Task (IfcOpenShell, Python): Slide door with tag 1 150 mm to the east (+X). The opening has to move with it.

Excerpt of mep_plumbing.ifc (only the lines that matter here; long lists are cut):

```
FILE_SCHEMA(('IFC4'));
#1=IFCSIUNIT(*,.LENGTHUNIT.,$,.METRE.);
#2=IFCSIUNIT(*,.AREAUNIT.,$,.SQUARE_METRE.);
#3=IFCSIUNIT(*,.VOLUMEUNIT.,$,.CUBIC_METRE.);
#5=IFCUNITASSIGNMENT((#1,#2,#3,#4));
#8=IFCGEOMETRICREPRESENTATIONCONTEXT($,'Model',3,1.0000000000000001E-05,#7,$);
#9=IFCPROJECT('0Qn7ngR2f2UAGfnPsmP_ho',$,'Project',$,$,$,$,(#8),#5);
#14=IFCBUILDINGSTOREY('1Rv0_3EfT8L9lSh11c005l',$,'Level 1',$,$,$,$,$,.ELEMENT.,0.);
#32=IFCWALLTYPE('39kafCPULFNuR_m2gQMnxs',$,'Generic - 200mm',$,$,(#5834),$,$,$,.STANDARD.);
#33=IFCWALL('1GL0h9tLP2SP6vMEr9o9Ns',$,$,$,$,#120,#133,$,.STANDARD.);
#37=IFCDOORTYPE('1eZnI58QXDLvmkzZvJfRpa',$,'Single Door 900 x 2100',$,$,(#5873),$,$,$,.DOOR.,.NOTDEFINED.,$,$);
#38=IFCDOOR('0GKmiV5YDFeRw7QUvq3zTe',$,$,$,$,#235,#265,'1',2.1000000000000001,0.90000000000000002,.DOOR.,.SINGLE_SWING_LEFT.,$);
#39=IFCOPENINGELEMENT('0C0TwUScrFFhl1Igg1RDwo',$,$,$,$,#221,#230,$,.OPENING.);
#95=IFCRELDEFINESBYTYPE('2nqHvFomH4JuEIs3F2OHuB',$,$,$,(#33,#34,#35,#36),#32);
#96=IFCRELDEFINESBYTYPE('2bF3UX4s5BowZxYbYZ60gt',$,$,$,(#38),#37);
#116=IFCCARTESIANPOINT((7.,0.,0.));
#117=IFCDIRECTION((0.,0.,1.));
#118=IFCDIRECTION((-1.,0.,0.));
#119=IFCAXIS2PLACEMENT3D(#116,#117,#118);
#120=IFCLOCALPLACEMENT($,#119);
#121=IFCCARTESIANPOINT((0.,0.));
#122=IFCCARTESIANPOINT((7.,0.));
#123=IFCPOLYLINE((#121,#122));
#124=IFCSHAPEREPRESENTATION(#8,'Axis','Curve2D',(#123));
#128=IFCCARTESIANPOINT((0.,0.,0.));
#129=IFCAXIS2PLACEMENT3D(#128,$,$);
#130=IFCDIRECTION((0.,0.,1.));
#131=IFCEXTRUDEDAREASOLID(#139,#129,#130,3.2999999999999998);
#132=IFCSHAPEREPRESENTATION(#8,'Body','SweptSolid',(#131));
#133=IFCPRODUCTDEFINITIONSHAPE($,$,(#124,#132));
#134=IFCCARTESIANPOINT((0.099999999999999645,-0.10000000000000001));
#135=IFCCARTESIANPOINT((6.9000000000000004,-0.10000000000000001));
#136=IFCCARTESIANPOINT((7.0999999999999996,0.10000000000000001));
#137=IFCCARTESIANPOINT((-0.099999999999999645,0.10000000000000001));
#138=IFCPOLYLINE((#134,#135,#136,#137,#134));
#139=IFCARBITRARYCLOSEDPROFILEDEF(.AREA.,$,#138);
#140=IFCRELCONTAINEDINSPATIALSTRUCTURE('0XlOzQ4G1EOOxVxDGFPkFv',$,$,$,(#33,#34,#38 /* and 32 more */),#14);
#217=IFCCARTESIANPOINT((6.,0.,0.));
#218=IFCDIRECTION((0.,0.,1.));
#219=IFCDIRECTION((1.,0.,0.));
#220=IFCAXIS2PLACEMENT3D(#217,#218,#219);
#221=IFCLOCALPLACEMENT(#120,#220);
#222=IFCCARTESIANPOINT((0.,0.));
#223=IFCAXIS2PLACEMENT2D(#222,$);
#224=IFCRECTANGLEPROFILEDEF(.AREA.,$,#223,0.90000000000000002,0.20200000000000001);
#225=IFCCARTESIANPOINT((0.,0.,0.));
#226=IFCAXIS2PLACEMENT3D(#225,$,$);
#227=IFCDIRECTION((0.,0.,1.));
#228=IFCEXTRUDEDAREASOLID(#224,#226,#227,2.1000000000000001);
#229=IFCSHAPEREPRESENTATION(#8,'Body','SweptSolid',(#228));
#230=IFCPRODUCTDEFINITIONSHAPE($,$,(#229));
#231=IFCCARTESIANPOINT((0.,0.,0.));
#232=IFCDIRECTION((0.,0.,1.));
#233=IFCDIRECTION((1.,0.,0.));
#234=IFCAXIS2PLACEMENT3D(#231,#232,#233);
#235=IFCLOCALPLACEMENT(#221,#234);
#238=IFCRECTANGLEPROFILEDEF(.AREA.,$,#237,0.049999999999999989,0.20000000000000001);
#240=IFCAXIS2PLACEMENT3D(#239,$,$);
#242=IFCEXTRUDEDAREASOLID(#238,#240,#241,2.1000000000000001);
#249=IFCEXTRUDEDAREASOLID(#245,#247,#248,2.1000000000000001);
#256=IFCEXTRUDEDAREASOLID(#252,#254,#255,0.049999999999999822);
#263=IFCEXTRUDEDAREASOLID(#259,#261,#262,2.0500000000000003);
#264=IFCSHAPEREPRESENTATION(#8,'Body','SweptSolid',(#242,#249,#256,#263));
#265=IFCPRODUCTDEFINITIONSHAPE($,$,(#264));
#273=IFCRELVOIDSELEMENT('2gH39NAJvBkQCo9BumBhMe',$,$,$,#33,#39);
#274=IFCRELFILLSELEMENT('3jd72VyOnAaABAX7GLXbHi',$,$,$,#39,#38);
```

```python
import ifcopenshell
import ifcopenshell.api.geometry
import ifcopenshell.util.placement

model = ifcopenshell.open("mep_plumbing.ifc")

door = model.by_id(38)
opening = door.FillsVoids[0].RelatingOpeningElement
wall = opening.VoidsElements[0].RelatingBuildingElement

wall_matrix = ifcopenshell.util.placement.get_local_placement(wall.ObjectPlacement)
shift = wall_matrix[:3, 0] * -0.15
before = ifcopenshell.util.placement.get_local_placement(door.ObjectPlacement)[:3, 3].copy()

# The door is placed relative to its opening, so it follows when the opening moves.
matrix = ifcopenshell.util.placement.get_local_placement(opening.ObjectPlacement)
matrix[:3, 3] += shift
ifcopenshell.api.geometry.edit_object_placement(
    model, product=opening, matrix=matrix, is_si=False, should_transform_children=True
)

after = ifcopenshell.util.placement.get_local_placement(door.ObjectPlacement)[:3, 3]
print("door moved by", (after - before).round(3) + 0.0)

model.write("mep_plumbing_edited.ifc")
```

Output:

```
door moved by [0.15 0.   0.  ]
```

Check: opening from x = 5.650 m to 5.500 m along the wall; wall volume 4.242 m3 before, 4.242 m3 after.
